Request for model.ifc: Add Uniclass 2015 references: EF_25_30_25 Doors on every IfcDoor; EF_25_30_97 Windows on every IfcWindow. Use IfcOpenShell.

First a look at what the model holds.

```python
import ifcopenshell

model = ifcopenshell.open("model.ifc")
print(model.schema)
print("classifications:", [c.Name for c in model.by_type("IfcClassification")])
for ifc_class in ("IfcDoor", "IfcRoof", "IfcStair", "IfcWall", "IfcWindow"):
    print(ifc_class, len(model.by_type(ifc_class)))
```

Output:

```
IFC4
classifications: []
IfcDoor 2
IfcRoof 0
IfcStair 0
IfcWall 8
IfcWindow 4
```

```python
import ifcopenshell
import ifcopenshell.api.classification

model = ifcopenshell.open("model.ifc")

system = ifcopenshell.api.classification.add_classification(model, classification="Uniclass 2015")

codes = {
    "IfcDoor": ("EF_25_30_25", "Doors"),
    "IfcWindow": ("EF_25_30_97", "Windows"),
}
for ifc_class, (code, name) in codes.items():
    products = model.by_type(ifc_class)
    ifcopenshell.api.classification.add_reference(
        model, products=products, classification=system, identification=code, name=name
    )
    print(code, len(products))

model.write("model_v2.ifc")
```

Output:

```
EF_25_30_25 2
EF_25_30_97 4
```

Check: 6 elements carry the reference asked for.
